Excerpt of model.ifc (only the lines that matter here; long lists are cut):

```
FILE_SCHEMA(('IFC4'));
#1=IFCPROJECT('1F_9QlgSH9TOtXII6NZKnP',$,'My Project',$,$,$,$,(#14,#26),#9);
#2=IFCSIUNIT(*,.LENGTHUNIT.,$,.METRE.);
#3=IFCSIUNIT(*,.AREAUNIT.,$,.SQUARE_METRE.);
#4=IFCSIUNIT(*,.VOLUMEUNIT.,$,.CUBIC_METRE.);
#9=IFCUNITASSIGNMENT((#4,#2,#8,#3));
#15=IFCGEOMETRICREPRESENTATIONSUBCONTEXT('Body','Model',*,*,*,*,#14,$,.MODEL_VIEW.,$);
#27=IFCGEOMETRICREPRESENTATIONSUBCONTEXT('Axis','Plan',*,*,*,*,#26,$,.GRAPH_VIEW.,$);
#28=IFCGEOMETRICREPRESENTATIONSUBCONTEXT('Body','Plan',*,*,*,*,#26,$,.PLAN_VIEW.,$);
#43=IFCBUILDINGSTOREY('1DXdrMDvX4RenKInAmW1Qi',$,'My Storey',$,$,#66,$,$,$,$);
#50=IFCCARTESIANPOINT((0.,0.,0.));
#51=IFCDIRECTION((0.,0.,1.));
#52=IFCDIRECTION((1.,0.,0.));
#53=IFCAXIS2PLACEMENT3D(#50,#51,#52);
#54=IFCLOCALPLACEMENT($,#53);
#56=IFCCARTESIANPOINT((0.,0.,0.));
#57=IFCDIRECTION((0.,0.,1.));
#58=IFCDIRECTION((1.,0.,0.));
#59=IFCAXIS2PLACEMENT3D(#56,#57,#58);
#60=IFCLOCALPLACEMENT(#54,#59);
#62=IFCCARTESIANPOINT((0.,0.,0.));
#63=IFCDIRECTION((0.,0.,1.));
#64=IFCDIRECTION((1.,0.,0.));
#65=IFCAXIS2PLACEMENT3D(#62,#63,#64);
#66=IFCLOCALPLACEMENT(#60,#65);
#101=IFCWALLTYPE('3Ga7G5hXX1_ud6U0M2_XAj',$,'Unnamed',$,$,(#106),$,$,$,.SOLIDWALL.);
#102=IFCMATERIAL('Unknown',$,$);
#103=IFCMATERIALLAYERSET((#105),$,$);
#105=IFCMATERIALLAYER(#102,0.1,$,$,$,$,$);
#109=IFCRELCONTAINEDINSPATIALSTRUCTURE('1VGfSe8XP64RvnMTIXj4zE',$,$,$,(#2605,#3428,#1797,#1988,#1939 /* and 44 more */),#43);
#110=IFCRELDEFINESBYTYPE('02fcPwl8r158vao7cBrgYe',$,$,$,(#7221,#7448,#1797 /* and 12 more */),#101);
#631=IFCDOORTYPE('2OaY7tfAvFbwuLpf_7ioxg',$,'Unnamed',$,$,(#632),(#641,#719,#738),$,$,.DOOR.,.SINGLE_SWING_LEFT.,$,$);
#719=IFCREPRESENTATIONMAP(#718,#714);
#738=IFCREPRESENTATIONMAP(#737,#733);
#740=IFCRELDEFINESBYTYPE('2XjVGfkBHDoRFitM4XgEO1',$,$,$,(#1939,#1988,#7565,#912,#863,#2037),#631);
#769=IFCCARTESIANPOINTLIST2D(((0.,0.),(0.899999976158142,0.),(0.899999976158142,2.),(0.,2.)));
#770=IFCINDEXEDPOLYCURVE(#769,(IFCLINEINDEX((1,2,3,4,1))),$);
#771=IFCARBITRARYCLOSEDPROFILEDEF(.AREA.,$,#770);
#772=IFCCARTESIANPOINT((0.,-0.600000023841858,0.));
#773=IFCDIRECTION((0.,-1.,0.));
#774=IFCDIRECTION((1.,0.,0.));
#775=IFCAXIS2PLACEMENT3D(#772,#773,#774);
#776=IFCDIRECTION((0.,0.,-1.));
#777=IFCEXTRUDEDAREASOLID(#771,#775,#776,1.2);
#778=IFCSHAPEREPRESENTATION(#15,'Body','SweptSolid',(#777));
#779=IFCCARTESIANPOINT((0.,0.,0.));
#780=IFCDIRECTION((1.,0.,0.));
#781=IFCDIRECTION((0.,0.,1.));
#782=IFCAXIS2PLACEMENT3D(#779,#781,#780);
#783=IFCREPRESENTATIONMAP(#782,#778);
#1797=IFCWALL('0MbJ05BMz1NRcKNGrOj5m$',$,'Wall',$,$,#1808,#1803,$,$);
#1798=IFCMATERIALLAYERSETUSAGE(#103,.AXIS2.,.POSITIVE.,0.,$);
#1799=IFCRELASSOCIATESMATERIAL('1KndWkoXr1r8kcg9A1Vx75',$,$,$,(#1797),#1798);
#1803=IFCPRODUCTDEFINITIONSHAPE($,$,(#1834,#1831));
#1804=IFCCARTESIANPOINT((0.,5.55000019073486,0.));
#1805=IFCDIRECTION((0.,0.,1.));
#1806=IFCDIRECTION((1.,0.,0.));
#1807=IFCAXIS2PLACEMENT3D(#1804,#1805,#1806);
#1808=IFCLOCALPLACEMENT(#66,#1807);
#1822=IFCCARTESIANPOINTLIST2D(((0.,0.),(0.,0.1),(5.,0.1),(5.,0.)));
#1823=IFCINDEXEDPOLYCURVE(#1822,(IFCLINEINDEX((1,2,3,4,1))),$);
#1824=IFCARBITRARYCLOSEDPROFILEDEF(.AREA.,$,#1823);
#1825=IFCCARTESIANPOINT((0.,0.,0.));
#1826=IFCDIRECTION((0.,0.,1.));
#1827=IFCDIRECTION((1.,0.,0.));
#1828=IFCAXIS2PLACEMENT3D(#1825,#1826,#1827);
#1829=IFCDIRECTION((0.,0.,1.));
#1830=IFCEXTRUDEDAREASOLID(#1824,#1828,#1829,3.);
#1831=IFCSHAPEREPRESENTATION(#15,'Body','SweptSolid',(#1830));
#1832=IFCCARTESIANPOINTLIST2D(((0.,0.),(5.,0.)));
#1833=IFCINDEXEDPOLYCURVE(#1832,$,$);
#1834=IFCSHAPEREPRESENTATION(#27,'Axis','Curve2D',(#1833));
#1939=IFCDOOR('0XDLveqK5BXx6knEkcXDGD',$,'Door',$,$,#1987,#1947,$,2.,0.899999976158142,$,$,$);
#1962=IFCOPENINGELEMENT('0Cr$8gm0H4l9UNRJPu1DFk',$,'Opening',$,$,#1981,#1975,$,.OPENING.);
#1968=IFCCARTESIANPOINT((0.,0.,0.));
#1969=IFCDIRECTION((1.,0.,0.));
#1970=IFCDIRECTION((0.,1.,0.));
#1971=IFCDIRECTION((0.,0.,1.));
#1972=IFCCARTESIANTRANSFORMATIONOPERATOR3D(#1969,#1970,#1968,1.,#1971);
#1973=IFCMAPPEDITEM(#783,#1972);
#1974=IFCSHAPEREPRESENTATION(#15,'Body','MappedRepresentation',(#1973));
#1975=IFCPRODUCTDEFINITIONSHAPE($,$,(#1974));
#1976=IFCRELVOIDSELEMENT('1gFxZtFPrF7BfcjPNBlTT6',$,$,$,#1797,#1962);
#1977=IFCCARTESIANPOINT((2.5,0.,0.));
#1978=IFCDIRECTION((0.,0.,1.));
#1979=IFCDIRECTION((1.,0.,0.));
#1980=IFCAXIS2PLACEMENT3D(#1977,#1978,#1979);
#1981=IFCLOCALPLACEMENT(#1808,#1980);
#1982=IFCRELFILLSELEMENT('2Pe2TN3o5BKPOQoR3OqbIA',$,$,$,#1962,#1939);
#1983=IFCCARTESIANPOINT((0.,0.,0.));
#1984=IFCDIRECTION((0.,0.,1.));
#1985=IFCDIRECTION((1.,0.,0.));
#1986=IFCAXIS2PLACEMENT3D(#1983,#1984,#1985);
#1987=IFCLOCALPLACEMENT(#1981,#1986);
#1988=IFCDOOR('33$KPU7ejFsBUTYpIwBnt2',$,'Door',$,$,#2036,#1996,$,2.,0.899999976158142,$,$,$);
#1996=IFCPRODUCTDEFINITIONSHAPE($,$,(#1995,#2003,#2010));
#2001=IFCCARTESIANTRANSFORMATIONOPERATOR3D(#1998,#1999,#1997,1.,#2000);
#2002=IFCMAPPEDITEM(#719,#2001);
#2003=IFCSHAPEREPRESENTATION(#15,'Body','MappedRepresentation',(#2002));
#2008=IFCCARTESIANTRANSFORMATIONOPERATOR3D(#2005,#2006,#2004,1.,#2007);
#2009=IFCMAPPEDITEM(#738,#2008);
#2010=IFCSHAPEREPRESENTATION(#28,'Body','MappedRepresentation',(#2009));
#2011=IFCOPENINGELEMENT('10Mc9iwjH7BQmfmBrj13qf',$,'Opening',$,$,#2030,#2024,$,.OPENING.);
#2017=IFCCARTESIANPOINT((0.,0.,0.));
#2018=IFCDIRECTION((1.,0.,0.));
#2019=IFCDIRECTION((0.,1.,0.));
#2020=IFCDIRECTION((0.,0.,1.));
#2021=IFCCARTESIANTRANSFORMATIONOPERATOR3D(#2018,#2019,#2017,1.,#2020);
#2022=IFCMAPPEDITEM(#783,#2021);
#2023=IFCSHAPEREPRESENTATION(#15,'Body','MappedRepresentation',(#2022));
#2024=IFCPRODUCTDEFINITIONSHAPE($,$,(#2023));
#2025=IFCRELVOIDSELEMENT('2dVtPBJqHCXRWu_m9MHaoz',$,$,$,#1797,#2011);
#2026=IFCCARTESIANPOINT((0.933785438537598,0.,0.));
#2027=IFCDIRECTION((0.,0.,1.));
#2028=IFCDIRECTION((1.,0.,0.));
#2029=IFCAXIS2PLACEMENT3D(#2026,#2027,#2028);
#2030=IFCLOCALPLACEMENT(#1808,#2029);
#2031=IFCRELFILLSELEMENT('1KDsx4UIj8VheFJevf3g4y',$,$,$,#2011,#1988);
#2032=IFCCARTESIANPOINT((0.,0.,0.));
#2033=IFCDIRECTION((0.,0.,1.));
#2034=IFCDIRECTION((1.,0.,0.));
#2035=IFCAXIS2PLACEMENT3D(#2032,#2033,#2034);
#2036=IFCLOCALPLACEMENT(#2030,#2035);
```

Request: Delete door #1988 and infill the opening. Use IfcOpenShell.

```python
import ifcopenshell
import ifcopenshell.api.feature
import ifcopenshell.api.root
import ifcopenshell.geom
import ifcopenshell.util.shape

model = ifcopenshell.open("model.ifc")
settings = ifcopenshell.geom.settings()


def volume(element):
    """Net volume in cubic metres, openings subtracted."""
    shape = ifcopenshell.geom.create_shape(settings, element)
    return ifcopenshell.util.shape.get_volume(shape.geometry)


door = model.by_id(1988)
opening = door.FillsVoids[0].RelatingOpeningElement
wall = opening.VoidsElements[0].RelatingBuildingElement
before = volume(wall)

ifcopenshell.api.root.remove_product(model, product=door)
ifcopenshell.api.feature.remove_feature(model, feature=opening)

after = volume(wall)

print(f"wall volume {before:.3f} -> {after:.3f} m3")

model.write("model_rev.ifc")
```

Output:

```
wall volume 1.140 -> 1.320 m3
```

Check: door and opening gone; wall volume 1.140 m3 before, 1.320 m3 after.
